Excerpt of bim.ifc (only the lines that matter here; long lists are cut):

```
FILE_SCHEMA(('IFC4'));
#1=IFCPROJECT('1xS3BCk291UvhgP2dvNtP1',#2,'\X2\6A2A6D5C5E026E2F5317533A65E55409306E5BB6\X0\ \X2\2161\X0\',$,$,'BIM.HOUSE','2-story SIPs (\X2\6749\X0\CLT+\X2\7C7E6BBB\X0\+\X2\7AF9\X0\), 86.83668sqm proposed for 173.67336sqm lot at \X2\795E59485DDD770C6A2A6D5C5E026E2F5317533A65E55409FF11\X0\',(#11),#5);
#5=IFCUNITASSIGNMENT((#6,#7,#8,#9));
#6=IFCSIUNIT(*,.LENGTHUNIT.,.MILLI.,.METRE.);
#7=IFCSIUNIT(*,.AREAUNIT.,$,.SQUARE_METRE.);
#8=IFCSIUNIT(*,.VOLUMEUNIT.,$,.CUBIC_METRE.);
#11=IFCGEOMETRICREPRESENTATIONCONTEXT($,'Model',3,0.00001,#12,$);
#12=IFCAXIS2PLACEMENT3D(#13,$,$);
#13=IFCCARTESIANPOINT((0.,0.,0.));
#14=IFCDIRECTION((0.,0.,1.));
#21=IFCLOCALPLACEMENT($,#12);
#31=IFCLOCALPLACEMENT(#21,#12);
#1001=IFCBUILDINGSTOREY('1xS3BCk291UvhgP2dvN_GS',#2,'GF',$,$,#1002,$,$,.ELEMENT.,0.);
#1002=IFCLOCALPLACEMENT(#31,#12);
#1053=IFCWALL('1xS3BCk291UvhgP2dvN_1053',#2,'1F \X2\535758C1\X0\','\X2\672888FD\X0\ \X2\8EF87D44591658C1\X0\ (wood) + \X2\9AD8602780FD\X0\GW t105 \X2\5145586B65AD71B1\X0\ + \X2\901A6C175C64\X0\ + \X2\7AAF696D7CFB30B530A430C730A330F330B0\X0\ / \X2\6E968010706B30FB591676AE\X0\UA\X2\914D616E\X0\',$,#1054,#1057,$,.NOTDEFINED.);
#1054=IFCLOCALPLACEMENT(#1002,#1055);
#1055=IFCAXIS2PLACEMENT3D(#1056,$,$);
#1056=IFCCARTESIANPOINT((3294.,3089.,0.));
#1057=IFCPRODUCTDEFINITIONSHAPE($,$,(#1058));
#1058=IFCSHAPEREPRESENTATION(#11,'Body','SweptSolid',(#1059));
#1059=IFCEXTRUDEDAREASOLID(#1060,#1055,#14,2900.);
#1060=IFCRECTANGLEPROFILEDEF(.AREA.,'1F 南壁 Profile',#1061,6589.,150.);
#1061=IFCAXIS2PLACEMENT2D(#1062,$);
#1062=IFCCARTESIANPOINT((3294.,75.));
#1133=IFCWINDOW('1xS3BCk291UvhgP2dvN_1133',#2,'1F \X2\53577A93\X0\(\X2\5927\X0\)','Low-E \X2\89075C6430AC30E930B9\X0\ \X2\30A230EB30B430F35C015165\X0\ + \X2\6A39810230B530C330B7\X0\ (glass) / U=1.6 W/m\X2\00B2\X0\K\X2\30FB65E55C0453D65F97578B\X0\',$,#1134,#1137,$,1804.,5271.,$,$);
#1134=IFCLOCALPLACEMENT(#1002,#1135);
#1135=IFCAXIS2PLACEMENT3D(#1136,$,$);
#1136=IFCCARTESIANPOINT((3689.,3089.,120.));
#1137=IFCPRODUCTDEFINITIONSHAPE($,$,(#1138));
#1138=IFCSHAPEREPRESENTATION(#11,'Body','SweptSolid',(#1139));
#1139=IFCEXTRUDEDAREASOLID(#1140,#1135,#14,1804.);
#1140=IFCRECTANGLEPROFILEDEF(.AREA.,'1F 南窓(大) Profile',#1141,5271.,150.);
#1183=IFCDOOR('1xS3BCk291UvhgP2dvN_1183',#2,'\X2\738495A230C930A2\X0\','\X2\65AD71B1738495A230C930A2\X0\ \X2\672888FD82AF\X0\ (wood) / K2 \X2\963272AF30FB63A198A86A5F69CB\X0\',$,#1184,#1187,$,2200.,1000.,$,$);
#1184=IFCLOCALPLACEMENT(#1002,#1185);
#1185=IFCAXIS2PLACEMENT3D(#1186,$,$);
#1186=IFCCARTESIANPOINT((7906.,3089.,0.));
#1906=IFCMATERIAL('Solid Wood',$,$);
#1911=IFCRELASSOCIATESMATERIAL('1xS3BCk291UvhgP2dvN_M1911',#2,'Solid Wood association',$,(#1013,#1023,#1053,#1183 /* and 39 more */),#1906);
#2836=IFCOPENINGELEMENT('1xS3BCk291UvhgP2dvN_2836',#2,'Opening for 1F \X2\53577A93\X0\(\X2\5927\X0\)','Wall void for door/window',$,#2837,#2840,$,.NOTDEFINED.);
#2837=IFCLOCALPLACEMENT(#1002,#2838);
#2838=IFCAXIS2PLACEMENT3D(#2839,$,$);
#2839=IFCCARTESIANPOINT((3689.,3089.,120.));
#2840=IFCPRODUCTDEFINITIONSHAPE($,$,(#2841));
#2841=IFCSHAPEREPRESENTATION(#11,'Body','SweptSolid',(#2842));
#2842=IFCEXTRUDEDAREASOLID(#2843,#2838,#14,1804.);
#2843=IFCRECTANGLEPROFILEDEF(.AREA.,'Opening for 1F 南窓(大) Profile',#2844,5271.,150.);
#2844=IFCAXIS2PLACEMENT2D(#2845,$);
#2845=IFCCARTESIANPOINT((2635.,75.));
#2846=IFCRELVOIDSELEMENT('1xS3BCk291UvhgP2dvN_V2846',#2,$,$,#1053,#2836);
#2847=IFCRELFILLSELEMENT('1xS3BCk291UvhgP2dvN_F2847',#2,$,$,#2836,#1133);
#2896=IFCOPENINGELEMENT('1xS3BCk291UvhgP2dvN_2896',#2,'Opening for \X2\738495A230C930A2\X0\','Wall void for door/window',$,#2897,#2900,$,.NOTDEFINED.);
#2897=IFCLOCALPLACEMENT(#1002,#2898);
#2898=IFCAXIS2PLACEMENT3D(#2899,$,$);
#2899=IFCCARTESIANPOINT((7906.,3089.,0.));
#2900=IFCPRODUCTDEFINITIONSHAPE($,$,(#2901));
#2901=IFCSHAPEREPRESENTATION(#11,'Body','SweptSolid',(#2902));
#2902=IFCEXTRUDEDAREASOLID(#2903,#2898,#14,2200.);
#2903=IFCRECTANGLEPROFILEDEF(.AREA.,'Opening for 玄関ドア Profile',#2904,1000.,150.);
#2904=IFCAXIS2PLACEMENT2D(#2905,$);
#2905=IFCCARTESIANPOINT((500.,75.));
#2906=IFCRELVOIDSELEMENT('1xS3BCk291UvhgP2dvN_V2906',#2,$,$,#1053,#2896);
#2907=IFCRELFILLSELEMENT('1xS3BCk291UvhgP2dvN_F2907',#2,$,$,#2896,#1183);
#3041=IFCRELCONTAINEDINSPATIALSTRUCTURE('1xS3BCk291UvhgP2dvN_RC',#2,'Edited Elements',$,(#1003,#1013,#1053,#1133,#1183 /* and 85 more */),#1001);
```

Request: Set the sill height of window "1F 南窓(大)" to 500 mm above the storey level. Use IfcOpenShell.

```python
import numpy as np
import ifcopenshell
import ifcopenshell.api.geometry
import ifcopenshell.geom
import ifcopenshell.util.element
import ifcopenshell.util.placement
import ifcopenshell.util.shape
import ifcopenshell.util.unit

model = ifcopenshell.open("bim.ifc")
unit_scale = ifcopenshell.util.unit.calculate_unit_scale(model)

window = model.by_guid("1xS3BCk291UvhgP2dvN_1133")
opening = window.FillsVoids[0].RelatingOpeningElement
storey = ifcopenshell.util.element.get_container(window, ifc_class="IfcBuildingStorey")
level = ifcopenshell.util.placement.get_local_placement(storey.ObjectPlacement)[2, 3]

# The opening's origin need not be at the sill, so measure its lowest point.
shape = ifcopenshell.geom.create_shape(ifcopenshell.geom.settings(), opening)
bottom = ifcopenshell.util.shape.get_shape_bottom_elevation(shape, shape.geometry) / unit_scale
dz = level + 0.5 / unit_scale - bottom

shift = np.array([0.0, 0.0, dz])
# The window is not placed relative to its opening, so move both.
for product in (opening, window):
    matrix = ifcopenshell.util.placement.get_local_placement(product.ObjectPlacement)
    matrix[:3, 3] += shift
    ifcopenshell.api.geometry.edit_object_placement(model, product=product, matrix=matrix, is_si=False)

print(f"moved by {dz * unit_scale:+.3f} m")

model.write("bim-out.ifc")
```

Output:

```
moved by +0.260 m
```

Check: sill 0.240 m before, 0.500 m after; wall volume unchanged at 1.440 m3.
